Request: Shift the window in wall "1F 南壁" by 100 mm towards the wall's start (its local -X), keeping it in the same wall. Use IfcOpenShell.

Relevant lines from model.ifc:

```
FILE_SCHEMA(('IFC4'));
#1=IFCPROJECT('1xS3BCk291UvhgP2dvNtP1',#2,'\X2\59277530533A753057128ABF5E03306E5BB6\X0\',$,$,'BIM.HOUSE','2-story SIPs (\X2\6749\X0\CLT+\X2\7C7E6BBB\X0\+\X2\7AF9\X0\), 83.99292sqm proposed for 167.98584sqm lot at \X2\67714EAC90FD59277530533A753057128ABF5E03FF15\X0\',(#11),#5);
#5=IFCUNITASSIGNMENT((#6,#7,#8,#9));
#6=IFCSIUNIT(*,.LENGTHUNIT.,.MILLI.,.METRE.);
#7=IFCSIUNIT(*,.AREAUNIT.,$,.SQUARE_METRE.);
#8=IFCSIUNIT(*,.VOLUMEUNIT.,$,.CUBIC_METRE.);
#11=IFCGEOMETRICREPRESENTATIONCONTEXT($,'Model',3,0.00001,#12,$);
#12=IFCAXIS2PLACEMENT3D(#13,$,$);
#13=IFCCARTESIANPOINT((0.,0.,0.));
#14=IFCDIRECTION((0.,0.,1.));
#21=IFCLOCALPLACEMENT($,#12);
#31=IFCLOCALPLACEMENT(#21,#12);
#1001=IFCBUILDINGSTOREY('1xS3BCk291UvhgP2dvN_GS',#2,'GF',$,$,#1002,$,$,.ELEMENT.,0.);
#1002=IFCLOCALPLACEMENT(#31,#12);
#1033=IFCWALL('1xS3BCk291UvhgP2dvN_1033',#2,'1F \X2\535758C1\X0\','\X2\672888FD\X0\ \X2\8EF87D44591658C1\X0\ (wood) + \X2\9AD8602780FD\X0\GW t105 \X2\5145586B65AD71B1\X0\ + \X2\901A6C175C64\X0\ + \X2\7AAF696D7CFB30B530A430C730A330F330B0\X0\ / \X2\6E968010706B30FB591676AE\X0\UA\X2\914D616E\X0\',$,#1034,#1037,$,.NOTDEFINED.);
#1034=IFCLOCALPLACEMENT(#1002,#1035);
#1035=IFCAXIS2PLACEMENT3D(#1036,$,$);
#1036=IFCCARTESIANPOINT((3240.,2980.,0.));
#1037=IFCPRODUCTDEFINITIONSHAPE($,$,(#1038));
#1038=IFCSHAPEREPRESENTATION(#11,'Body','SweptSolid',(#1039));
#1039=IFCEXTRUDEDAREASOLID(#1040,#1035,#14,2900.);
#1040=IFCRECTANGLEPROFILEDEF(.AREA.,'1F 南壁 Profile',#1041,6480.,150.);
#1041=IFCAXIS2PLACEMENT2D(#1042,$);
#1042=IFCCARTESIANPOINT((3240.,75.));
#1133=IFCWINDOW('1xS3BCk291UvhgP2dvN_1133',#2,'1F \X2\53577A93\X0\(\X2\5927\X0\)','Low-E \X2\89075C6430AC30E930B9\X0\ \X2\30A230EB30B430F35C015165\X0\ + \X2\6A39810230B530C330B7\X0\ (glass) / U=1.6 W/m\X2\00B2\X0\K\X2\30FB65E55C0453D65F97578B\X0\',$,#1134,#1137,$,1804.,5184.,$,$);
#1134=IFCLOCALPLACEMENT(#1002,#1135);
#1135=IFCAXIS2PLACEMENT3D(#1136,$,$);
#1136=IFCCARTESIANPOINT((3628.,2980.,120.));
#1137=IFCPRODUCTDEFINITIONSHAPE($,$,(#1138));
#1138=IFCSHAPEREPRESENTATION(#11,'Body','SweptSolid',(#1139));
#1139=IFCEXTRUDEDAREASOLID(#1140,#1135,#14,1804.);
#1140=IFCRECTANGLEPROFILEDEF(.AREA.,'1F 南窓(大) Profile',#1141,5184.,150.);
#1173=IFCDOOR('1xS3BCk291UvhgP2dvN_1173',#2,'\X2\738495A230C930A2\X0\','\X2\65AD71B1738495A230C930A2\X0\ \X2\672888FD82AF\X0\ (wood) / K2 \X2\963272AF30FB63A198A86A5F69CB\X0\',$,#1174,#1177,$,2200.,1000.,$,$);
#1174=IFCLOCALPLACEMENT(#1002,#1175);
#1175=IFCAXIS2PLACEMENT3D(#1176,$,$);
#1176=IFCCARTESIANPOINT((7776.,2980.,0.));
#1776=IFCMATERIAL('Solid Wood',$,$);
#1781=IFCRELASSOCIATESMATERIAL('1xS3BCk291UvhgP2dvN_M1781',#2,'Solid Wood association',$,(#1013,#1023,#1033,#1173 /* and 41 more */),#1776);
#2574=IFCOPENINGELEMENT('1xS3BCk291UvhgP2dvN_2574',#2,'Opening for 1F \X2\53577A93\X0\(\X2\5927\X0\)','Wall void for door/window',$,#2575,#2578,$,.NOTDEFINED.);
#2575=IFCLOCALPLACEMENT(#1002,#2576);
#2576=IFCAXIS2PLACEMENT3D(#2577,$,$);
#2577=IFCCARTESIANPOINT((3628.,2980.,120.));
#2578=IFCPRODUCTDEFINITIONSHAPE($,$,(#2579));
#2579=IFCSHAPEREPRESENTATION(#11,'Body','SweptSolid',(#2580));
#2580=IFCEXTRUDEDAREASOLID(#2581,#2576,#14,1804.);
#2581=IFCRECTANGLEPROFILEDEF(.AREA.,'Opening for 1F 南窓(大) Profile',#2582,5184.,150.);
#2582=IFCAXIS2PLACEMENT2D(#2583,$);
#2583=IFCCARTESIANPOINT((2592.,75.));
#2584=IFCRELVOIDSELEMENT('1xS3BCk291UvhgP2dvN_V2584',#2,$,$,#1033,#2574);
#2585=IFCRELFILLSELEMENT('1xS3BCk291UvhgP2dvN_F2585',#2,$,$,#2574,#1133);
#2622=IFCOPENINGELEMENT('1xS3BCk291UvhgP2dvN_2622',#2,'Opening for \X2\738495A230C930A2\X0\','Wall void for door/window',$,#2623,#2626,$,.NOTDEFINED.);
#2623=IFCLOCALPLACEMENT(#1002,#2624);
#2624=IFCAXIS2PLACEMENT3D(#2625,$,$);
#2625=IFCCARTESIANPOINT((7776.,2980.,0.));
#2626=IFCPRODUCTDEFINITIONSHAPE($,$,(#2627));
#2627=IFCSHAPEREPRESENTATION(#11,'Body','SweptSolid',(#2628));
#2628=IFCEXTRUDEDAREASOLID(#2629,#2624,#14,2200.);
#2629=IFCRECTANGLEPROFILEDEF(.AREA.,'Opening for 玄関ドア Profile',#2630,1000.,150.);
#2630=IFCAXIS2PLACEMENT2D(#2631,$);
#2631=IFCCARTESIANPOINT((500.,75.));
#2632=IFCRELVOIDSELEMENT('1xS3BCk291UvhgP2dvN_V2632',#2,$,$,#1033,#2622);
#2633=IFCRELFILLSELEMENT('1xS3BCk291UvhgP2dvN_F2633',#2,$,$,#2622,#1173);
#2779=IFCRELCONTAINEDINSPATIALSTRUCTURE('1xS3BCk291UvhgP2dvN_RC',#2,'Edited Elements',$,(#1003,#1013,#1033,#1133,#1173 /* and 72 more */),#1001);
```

```python
import ifcopenshell
import ifcopenshell.api.geometry
import ifcopenshell.util.placement

model = ifcopenshell.open("model.ifc")

window = model.by_id(1133)
opening = window.FillsVoids[0].RelatingOpeningElement
wall = opening.VoidsElements[0].RelatingBuildingElement

wall_matrix = ifcopenshell.util.placement.get_local_placement(wall.ObjectPlacement)
shift = wall_matrix[:3, 0] * -100.0
before = ifcopenshell.util.placement.get_local_placement(window.ObjectPlacement)[:3, 3].copy()

# The window is not placed relative to its opening, so move both.
for product in (opening, window):
    matrix = ifcopenshell.util.placement.get_local_placement(product.ObjectPlacement)
    matrix[:3, 3] += shift
    ifcopenshell.api.geometry.edit_object_placement(model, product=product, matrix=matrix, is_si=False)

after = ifcopenshell.util.placement.get_local_placement(window.ObjectPlacement)[:3, 3]
print("window moved by", (after - before).round(3) + 0.0)

model.write("model_rev.ifc")
```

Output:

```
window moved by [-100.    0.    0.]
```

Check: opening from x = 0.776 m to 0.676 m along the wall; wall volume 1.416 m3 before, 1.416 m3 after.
